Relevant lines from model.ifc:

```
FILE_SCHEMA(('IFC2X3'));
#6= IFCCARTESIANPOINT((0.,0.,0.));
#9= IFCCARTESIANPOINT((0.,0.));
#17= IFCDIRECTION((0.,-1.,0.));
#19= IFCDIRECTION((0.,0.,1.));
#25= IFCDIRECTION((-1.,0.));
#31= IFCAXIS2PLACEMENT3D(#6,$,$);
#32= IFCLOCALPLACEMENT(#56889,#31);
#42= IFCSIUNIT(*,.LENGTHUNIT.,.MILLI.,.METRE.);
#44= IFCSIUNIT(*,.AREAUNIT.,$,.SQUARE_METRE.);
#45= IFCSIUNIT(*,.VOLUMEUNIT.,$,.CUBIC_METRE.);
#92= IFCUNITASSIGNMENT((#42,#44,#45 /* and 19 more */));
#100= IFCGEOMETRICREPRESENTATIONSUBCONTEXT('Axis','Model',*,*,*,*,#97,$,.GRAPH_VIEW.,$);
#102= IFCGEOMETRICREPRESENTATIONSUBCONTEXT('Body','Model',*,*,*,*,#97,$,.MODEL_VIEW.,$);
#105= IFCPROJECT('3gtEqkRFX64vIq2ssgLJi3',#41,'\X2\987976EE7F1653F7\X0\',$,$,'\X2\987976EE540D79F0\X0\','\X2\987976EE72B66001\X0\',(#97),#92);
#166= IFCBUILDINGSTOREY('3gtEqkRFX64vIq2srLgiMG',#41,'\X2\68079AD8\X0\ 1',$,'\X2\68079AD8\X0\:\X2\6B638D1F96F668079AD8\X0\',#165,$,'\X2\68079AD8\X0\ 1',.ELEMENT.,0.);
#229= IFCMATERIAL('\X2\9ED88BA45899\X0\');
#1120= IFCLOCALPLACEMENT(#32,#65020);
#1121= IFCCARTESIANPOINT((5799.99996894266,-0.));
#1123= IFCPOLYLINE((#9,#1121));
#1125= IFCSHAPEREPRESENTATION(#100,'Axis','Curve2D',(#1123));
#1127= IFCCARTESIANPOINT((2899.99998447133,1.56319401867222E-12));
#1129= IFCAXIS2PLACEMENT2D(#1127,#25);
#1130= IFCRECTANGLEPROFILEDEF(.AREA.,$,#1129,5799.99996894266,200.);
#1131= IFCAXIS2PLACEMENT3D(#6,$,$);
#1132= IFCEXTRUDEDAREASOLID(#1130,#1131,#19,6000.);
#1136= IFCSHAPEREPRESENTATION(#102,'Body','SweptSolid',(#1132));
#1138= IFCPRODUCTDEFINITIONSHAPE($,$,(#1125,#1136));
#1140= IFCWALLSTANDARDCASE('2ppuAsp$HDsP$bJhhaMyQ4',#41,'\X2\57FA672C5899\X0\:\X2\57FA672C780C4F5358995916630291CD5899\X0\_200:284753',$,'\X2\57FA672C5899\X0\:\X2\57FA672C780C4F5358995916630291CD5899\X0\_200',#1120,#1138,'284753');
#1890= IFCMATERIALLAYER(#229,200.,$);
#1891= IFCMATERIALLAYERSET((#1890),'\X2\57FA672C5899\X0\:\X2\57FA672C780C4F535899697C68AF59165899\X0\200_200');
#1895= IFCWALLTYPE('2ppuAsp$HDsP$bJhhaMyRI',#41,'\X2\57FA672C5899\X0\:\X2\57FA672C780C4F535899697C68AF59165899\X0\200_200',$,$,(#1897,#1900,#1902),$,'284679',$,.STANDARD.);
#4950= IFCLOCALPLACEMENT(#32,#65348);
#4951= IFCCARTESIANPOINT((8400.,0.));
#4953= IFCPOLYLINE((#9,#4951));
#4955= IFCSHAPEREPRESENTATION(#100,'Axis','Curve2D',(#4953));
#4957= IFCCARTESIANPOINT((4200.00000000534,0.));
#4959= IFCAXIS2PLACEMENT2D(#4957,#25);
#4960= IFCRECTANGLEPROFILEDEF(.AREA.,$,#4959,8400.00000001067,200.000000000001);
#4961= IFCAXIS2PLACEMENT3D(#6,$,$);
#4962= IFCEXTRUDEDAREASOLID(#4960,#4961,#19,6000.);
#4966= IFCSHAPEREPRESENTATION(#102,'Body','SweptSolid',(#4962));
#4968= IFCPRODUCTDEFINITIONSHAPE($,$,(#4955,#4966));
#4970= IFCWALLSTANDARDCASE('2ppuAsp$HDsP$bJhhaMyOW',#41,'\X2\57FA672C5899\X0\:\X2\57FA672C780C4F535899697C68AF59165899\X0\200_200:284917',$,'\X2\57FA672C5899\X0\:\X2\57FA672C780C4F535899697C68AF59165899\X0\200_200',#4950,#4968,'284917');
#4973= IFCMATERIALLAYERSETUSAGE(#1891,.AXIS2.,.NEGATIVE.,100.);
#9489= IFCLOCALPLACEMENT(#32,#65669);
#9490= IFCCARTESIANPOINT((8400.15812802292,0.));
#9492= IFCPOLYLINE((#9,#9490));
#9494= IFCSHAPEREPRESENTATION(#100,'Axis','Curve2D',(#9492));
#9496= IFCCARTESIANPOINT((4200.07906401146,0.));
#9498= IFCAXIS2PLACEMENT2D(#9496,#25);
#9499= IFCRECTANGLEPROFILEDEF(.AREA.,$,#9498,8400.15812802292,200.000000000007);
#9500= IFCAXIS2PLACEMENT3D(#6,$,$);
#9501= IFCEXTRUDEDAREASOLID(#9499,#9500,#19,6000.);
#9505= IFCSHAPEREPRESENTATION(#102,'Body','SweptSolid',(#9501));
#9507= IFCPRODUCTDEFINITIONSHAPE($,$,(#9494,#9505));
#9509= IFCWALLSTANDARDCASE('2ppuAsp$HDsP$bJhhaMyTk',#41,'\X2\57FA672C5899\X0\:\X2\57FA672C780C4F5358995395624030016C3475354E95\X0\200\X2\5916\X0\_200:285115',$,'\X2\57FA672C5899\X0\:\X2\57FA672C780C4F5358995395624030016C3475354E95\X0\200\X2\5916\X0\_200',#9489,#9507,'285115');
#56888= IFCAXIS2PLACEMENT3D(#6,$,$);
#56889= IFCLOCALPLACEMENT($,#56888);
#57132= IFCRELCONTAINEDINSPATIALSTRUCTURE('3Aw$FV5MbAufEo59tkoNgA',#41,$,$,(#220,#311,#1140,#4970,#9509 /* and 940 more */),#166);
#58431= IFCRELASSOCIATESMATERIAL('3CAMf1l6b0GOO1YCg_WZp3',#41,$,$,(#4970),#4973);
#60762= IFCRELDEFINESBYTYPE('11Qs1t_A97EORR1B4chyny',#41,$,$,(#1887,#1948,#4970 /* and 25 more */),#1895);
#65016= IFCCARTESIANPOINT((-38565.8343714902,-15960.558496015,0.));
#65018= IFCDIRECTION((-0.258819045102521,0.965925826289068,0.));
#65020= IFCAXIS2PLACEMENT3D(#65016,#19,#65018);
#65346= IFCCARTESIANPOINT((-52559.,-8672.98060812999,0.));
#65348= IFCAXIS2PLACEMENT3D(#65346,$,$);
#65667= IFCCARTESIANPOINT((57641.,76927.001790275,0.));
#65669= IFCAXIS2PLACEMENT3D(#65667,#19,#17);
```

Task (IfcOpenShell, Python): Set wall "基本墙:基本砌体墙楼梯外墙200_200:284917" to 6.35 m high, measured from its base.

```python
import ifcopenshell
import ifcopenshell.geom
import ifcopenshell.util.representation
import ifcopenshell.util.shape

model = ifcopenshell.open("model.ifc")
settings = ifcopenshell.geom.settings()


def volume(element):
    """Net volume in cubic metres, openings subtracted."""
    shape = ifcopenshell.geom.create_shape(settings, element)
    return ifcopenshell.util.shape.get_volume(shape.geometry)


wall = model.by_guid("2ppuAsp$HDsP$bJhhaMyOW")
before = volume(wall)

body = ifcopenshell.util.representation.get_representation(wall, "Model", "Body")
solid = body.Items[0]
old_height = solid.Depth
solid.Depth = 6350.0
after = volume(wall)

print(f"height {old_height:g} -> {solid.Depth:g}, volume {before:.3f} -> {after:.3f} m3")

model.write("model_edited.ifc")
```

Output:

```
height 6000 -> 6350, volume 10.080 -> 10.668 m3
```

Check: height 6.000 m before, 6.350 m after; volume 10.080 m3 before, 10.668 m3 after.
